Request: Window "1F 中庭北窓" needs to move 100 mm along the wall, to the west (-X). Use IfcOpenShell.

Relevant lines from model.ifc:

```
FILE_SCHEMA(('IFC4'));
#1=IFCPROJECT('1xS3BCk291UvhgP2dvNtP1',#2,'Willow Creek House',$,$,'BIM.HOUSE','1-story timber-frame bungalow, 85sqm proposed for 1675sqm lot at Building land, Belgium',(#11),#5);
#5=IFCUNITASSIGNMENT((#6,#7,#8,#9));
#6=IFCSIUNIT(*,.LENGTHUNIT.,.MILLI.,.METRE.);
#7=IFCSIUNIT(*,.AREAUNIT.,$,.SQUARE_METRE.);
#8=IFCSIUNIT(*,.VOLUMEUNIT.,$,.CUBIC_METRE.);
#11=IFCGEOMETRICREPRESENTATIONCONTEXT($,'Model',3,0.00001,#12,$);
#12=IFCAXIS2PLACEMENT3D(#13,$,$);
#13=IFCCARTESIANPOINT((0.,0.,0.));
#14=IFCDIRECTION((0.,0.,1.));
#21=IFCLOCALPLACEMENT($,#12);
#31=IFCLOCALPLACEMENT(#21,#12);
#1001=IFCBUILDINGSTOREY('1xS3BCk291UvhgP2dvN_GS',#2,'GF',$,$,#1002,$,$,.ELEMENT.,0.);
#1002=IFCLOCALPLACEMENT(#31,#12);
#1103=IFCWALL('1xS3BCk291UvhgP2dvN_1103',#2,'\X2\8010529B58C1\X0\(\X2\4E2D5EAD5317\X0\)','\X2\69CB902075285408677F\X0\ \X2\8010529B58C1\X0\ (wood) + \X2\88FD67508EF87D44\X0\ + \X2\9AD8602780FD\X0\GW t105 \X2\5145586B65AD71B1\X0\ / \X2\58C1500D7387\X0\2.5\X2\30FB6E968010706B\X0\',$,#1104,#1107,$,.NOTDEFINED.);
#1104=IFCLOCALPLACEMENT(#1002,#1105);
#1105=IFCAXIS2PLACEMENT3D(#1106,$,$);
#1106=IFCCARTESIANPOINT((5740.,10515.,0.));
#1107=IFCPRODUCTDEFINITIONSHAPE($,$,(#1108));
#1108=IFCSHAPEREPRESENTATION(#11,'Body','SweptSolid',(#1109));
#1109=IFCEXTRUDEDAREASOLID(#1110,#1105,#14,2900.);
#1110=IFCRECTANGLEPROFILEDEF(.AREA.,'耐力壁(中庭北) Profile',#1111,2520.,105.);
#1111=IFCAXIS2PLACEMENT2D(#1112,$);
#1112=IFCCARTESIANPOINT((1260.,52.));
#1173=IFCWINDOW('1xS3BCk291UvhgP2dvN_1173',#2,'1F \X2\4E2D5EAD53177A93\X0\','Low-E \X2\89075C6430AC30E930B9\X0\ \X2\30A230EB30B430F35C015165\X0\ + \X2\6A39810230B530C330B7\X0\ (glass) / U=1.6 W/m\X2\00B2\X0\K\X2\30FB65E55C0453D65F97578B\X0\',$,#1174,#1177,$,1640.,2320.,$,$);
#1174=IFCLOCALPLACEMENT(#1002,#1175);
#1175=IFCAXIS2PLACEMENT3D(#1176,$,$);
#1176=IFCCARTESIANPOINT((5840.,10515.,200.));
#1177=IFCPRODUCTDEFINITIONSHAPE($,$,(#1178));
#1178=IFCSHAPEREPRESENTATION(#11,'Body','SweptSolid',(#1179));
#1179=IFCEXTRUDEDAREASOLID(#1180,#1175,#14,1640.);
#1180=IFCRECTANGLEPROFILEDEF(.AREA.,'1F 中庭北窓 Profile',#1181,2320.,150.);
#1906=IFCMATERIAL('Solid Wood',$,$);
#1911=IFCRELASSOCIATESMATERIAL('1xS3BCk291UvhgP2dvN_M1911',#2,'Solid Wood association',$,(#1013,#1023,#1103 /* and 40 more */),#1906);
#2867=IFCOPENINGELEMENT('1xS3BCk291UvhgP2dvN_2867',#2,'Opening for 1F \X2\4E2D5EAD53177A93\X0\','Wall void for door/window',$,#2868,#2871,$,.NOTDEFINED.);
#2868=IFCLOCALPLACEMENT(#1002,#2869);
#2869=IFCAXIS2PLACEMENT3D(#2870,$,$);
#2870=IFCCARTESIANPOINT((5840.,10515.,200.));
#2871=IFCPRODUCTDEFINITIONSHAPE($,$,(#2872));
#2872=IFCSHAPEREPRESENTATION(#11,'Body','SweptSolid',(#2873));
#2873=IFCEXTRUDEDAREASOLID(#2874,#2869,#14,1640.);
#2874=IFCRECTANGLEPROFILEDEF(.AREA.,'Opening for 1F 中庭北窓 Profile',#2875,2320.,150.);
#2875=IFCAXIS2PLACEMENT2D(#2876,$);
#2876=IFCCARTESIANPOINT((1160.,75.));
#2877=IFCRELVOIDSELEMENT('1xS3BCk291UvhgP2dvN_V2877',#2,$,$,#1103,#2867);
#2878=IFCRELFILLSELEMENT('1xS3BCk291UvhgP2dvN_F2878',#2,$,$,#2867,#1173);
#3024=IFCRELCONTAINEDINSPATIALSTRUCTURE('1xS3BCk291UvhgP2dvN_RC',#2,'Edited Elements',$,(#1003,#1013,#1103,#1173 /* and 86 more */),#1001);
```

```python
import ifcopenshell
import ifcopenshell.api.geometry
import ifcopenshell.util.placement
import ifcopenshell.util.unit

model = ifcopenshell.open("model.ifc")
unit_scale = ifcopenshell.util.unit.calculate_unit_scale(model)

window = model.by_guid("1xS3BCk291UvhgP2dvN_1173")
opening = window.FillsVoids[0].RelatingOpeningElement
wall = opening.VoidsElements[0].RelatingBuildingElement

wall_matrix = ifcopenshell.util.placement.get_local_placement(wall.ObjectPlacement)
shift = wall_matrix[:3, 0] * -0.1 / unit_scale
before = ifcopenshell.util.placement.get_local_placement(window.ObjectPlacement)[:3, 3].copy()

# The window is not placed relative to its opening, so move both.
for product in (opening, window):
    matrix = ifcopenshell.util.placement.get_local_placement(product.ObjectPlacement)
    matrix[:3, 3] += shift
    ifcopenshell.api.geometry.edit_object_placement(model, product=product, matrix=matrix, is_si=False)

after = ifcopenshell.util.placement.get_local_placement(window.ObjectPlacement)[:3, 3]
print("window moved by", (after - before).round(3) + 0.0)

model.write("model_updated.ifc")
```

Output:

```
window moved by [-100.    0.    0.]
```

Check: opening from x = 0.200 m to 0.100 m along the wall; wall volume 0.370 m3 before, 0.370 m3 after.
